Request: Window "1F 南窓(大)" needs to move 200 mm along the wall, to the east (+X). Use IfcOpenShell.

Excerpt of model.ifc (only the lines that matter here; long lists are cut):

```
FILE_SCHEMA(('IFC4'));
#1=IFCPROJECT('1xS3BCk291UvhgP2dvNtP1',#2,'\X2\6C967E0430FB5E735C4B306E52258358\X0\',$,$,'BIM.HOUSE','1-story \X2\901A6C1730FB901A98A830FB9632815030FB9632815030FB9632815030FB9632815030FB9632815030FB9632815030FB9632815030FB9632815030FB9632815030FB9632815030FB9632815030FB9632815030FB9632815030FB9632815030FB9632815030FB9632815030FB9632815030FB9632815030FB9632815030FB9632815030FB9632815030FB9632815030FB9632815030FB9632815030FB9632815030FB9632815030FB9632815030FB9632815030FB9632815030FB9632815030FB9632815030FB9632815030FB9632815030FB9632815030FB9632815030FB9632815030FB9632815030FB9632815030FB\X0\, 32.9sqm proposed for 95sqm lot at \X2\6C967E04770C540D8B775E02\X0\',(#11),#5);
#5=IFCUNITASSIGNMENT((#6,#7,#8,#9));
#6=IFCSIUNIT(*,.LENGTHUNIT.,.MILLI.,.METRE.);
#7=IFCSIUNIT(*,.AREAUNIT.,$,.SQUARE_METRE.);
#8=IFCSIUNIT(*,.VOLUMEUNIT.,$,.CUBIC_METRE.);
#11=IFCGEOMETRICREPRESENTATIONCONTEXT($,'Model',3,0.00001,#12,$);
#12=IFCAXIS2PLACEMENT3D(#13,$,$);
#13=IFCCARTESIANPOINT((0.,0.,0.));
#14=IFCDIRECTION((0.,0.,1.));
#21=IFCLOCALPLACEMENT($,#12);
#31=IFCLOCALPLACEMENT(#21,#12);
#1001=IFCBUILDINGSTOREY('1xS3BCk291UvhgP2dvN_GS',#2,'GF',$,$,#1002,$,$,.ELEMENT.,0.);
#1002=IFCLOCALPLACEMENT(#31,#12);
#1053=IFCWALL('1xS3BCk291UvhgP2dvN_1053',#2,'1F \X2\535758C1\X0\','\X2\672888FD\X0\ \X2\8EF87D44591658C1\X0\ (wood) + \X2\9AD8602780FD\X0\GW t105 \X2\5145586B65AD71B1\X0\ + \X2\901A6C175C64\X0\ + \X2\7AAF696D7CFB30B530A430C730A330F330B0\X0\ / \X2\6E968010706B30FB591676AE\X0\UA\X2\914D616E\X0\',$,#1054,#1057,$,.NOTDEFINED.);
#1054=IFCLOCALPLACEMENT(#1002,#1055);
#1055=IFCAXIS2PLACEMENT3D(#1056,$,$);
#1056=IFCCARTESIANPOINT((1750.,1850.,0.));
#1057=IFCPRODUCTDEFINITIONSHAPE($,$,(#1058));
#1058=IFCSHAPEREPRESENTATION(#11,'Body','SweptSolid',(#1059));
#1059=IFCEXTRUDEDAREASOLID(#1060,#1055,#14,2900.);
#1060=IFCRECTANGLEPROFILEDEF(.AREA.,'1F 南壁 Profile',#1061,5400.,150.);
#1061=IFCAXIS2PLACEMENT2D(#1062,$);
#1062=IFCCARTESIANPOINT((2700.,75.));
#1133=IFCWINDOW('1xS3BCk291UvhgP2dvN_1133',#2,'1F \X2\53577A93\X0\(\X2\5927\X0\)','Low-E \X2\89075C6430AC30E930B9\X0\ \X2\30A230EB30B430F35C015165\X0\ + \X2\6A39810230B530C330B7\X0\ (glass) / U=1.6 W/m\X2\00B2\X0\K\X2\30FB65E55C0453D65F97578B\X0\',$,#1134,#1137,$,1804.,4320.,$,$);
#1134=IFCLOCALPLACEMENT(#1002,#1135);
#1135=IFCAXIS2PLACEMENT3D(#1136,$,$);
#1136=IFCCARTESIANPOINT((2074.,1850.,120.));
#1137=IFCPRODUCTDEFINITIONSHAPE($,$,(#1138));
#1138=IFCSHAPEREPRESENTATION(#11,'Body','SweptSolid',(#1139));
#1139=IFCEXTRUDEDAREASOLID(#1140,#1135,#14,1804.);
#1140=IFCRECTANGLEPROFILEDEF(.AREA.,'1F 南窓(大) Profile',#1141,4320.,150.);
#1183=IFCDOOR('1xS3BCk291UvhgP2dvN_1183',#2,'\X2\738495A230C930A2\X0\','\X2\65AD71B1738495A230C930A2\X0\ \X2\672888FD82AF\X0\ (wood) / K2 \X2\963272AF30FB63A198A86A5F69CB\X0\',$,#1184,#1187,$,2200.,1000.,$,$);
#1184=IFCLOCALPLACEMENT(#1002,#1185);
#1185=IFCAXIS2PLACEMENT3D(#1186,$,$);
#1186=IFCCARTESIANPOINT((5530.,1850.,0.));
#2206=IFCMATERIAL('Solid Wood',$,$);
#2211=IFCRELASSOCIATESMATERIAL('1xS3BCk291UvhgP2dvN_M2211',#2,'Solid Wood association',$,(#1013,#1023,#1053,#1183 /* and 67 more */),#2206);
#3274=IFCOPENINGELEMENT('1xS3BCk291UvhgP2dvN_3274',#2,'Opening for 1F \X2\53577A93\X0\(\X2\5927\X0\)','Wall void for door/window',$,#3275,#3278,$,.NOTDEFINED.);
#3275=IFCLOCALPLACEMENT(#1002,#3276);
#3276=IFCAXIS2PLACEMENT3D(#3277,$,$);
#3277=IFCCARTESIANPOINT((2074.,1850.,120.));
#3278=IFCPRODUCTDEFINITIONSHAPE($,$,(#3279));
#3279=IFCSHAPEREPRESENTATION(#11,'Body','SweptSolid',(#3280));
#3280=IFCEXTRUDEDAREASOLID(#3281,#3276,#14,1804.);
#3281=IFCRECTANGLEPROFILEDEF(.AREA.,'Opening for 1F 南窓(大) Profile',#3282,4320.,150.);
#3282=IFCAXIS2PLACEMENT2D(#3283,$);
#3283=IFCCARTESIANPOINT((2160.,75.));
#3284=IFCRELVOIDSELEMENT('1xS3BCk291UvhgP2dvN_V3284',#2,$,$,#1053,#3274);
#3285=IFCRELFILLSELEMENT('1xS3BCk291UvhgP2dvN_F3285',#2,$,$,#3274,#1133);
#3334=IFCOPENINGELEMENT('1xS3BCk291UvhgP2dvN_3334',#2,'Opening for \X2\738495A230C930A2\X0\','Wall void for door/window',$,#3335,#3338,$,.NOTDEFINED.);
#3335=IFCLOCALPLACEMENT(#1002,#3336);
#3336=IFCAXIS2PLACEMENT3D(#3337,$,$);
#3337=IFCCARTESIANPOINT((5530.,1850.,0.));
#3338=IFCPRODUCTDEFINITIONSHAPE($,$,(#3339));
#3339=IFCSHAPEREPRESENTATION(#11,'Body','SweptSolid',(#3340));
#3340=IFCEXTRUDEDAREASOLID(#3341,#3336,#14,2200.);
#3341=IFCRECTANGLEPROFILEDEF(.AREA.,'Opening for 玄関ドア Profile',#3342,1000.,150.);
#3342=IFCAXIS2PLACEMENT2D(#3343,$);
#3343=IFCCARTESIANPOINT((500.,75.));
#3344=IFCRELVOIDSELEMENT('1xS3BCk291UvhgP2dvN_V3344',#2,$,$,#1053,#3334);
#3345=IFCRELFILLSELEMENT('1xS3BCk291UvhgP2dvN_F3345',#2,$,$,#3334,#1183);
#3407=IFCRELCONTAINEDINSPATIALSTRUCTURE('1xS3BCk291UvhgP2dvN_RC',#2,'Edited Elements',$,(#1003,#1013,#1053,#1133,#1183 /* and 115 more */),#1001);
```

```python
import ifcopenshell
import ifcopenshell.api.geometry
import ifcopenshell.util.placement

model = ifcopenshell.open("model.ifc")

window = model.by_id(1133)
opening = window.FillsVoids[0].RelatingOpeningElement
wall = opening.VoidsElements[0].RelatingBuildingElement

wall_matrix = ifcopenshell.util.placement.get_local_placement(wall.ObjectPlacement)
shift = wall_matrix[:3, 0] * 200.0
before = ifcopenshell.util.placement.get_local_placement(window.ObjectPlacement)[:3, 3].copy()

# The window is not placed relative to its opening, so move both.
for product in (opening, window):
    matrix = ifcopenshell.util.placement.get_local_placement(product.ObjectPlacement)
    matrix[:3, 3] += shift
    ifcopenshell.api.geometry.edit_object_placement(model, product=product, matrix=matrix, is_si=False)

after = ifcopenshell.util.placement.get_local_placement(window.ObjectPlacement)[:3, 3]
print("window moved by", (after - before).round(3) + 0.0)

model.write("model_v2.ifc")
```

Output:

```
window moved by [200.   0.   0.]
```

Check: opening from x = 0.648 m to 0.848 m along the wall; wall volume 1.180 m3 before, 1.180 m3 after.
